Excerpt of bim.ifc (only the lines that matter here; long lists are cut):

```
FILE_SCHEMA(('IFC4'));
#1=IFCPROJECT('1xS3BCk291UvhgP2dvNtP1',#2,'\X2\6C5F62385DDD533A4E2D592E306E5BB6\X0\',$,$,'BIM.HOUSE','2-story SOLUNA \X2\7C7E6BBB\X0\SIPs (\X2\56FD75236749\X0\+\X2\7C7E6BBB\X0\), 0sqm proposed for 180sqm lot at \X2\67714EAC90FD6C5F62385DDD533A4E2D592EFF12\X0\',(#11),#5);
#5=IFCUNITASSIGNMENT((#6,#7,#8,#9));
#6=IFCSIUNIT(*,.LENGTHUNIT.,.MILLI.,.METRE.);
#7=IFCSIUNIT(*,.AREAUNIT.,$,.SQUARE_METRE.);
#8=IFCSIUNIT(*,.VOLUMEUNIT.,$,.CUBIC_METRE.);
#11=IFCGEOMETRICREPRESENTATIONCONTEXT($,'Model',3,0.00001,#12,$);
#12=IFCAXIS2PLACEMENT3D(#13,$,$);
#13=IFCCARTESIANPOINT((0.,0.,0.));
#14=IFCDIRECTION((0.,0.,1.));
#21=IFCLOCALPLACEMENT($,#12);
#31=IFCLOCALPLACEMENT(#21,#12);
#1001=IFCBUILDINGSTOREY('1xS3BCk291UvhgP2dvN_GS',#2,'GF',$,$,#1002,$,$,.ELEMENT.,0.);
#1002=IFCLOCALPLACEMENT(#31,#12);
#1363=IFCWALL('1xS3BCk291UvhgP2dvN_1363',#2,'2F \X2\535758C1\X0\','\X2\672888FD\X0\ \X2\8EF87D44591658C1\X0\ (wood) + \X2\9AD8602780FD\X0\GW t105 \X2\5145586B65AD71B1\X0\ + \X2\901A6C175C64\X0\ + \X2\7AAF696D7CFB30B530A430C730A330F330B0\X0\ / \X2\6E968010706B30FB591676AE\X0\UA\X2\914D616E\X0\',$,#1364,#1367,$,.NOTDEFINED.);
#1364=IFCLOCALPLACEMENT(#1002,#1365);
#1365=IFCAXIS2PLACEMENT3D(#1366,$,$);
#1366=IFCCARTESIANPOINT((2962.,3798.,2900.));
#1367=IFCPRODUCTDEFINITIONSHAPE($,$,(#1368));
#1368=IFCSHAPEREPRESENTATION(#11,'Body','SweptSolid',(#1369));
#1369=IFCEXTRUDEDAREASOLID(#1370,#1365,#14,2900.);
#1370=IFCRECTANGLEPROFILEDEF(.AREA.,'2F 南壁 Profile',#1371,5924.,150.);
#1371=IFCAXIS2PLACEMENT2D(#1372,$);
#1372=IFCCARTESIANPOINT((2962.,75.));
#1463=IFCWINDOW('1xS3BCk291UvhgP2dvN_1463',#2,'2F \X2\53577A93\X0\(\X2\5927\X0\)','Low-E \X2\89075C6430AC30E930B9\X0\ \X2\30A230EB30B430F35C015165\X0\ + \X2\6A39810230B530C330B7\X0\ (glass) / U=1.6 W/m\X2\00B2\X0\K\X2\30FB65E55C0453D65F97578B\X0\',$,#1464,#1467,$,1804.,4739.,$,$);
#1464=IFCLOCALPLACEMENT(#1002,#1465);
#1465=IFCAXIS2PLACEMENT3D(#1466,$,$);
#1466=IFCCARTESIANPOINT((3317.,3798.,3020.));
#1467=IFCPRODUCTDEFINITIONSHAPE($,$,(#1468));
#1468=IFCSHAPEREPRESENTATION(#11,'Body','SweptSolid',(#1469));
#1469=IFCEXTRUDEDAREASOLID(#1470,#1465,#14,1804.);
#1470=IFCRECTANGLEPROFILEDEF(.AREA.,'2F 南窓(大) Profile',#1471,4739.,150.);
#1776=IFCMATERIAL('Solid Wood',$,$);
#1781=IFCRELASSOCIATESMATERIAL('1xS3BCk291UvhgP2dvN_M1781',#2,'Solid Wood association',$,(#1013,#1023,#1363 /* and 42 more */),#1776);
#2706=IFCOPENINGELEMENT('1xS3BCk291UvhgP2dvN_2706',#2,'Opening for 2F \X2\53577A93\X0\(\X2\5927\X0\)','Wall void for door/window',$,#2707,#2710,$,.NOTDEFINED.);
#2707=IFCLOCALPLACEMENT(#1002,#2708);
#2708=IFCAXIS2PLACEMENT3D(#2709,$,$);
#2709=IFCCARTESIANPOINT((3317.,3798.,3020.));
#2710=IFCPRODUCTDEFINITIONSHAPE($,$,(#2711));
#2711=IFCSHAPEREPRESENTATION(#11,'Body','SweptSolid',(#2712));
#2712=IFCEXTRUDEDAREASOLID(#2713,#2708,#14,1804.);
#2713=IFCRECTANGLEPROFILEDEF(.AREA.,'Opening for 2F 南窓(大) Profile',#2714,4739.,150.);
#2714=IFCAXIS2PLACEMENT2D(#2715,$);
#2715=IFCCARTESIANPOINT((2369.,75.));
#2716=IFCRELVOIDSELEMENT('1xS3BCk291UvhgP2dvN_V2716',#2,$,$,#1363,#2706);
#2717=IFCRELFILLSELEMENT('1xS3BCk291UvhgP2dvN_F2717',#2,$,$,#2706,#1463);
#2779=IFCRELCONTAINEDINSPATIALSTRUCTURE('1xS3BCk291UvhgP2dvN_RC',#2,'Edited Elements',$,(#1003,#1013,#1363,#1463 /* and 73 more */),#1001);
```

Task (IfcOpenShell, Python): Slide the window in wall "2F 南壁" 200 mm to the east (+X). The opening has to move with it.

```python
import ifcopenshell
import ifcopenshell.api.geometry
import ifcopenshell.util.placement
import ifcopenshell.util.unit

model = ifcopenshell.open("bim.ifc")
unit_scale = ifcopenshell.util.unit.calculate_unit_scale(model)

window = model.by_guid("1xS3BCk291UvhgP2dvN_1463")
opening = window.FillsVoids[0].RelatingOpeningElement
wall = opening.VoidsElements[0].RelatingBuildingElement

wall_matrix = ifcopenshell.util.placement.get_local_placement(wall.ObjectPlacement)
shift = wall_matrix[:3, 0] * 0.2 / unit_scale
before = ifcopenshell.util.placement.get_local_placement(window.ObjectPlacement)[:3, 3].copy()

# The window is not placed relative to its opening, so move both.
for product in (opening, window):
    matrix = ifcopenshell.util.placement.get_local_placement(product.ObjectPlacement)
    matrix[:3, 3] += shift
    ifcopenshell.api.geometry.edit_object_placement(model, product=product, matrix=matrix, is_si=False)

after = ifcopenshell.util.placement.get_local_placement(window.ObjectPlacement)[:3, 3]
print("window moved by", (after - before).round(3) + 0.0)

model.write("bim_updated.ifc")
```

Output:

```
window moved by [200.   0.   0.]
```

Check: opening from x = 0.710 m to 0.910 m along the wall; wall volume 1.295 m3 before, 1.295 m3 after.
